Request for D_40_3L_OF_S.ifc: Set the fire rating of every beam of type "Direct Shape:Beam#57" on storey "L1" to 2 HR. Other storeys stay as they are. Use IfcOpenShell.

First a look at what the model holds.

```python
import ifcopenshell
import ifcopenshell.util.element

model = ifcopenshell.open("D_40_3L_OF_S.ifc")
print(model.schema)
storey = next(s for s in model.by_type("IfcBuildingStorey") if s.Name == "L1")
beams = [e for e in ifcopenshell.util.element.get_decomposition(storey) if e.is_a("IfcBeam")]
seen = {}
for e in beams:
    element_type = ifcopenshell.util.element.get_type(e)
    key = (element_type.Name if element_type != e and element_type else None, ifcopenshell.util.element.get_pset(e, "Pset_BeamCommon", "FireRating"))
    seen[key] = seen.get(key, 0) + 1
for (name, value), count in sorted(seen.items(), key=str):
    print(count, "x", name, "|", value)
```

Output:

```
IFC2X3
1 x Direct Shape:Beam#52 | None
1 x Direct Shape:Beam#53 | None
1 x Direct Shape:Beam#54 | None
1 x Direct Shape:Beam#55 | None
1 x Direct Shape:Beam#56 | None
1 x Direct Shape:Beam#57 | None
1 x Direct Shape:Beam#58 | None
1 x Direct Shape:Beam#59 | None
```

```python
import ifcopenshell
import ifcopenshell.api.pset
import ifcopenshell.util.element

model = ifcopenshell.open("D_40_3L_OF_S.ifc")

storey = next(s for s in model.by_type("IfcBuildingStorey") if s.Name == "L1")
beams = [e for e in ifcopenshell.util.element.get_decomposition(storey) if e.is_a("IfcBeam")]

count = 0
for e in beams:
    element_type = ifcopenshell.util.element.get_type(e)
    if element_type in (None, e) or element_type.Name != "Direct Shape:Beam#57":
        continue
    # add_pset returns the element's existing set when there is one.
    pset = ifcopenshell.api.pset.add_pset(model, product=e, name="Pset_BeamCommon")
    ifcopenshell.api.pset.edit_pset(model, pset=pset, properties={"FireRating": "2 HR"})
    count += 1

print(count, "beams updated")

model.write("D_40_3L_OF_S_updated.ifc")
```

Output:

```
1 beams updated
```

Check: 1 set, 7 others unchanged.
